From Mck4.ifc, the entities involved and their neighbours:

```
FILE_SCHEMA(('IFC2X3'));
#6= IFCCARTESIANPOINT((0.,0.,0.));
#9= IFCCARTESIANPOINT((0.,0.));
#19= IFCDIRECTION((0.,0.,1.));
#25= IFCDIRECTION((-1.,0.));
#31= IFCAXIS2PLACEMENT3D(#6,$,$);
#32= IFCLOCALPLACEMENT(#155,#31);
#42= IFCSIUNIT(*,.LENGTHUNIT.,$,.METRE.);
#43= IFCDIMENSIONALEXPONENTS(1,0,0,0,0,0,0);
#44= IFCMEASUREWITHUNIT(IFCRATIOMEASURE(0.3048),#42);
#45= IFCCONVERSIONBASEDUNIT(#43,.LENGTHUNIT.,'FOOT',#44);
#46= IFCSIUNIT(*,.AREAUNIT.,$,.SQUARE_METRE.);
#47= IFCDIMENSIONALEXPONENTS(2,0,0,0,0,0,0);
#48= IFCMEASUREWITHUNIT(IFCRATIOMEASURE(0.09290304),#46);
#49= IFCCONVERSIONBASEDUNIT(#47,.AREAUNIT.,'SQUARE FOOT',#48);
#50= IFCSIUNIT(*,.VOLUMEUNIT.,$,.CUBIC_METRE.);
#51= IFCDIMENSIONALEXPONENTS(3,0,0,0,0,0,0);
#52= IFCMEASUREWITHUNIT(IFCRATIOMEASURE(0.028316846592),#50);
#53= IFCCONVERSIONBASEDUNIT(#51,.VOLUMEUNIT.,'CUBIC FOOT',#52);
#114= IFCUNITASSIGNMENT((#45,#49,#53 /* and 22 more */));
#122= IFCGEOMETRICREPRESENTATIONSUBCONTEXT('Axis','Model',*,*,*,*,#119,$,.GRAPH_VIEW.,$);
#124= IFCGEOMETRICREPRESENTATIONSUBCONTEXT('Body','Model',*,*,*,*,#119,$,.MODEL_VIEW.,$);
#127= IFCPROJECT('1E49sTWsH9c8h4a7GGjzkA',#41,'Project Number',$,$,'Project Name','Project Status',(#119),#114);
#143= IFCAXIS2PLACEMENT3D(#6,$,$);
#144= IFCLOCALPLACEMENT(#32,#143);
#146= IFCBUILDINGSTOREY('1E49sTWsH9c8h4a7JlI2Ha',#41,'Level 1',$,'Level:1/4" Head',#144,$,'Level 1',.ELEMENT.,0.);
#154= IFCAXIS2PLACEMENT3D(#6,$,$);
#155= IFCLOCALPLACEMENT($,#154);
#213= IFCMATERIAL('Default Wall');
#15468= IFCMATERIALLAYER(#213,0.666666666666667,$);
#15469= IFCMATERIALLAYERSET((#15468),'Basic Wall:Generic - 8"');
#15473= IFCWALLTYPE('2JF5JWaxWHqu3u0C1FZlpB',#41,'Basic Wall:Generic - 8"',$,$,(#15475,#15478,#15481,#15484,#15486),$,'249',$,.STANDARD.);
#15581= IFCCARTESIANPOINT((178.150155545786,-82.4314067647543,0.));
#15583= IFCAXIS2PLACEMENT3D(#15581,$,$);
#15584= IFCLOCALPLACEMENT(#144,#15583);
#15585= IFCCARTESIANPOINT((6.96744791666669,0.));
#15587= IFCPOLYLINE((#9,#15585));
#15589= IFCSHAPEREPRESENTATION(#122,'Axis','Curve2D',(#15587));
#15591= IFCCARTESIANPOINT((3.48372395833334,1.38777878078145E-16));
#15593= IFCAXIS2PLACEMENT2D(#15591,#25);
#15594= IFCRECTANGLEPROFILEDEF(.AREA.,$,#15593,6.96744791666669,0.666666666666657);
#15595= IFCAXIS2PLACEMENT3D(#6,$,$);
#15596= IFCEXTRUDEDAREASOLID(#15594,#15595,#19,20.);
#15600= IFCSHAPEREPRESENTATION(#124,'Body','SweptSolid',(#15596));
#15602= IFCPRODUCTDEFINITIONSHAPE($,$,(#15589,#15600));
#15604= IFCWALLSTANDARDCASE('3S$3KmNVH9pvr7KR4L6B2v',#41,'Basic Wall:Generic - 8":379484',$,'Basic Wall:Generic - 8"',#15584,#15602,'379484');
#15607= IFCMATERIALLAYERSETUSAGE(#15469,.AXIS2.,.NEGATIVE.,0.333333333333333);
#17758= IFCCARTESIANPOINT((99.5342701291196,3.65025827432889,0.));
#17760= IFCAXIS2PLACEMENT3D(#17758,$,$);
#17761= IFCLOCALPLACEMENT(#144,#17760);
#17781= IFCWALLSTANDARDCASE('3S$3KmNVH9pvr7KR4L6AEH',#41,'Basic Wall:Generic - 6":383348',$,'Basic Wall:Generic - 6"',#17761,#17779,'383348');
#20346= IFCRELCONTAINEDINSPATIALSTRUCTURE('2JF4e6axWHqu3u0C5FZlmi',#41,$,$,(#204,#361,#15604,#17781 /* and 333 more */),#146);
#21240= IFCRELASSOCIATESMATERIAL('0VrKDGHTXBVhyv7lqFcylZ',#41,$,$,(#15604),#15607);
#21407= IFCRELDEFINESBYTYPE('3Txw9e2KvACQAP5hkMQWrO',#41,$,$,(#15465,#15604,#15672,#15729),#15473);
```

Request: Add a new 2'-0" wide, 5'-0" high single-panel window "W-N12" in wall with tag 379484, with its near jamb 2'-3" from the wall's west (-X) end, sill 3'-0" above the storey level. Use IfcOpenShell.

```python
import numpy as np
import ifcopenshell
import ifcopenshell.api.feature
import ifcopenshell.api.geometry
import ifcopenshell.api.root
import ifcopenshell.api.spatial
import ifcopenshell.api.type
import ifcopenshell.geom
import ifcopenshell.util.element
import ifcopenshell.util.placement
import ifcopenshell.util.representation
import ifcopenshell.util.shape
import ifcopenshell.util.unit

model = ifcopenshell.open("Mck4.ifc")
unit_scale = ifcopenshell.util.unit.calculate_unit_scale(model)
settings = ifcopenshell.geom.settings()


def volume(element):
    """Net volume in cubic metres, openings subtracted."""
    shape = ifcopenshell.geom.create_shape(settings, element)
    return ifcopenshell.util.shape.get_volume(shape.geometry)


wall = model.by_id(15604)
storey = ifcopenshell.util.element.get_container(wall, ifc_class="IfcBuildingStorey")
context = ifcopenshell.util.representation.get_context(model, "Model", "Body", "MODEL_VIEW")
before = volume(wall)

width, height, from_end, sill = 0.6096, 1.524, 0.6858, 0.9144  # metres

# The wall runs along its own X axis, and the end named is its -X end.
wall_shape = ifcopenshell.geom.create_shape(settings, wall)
x, y, z = ifcopenshell.util.shape.get_vertices(wall_shape.geometry).T
start = x.min() + from_end
face, thickness = float(y.min()), float(y.max() - y.min())
wall_matrix = ifcopenshell.util.placement.get_local_placement(wall.ObjectPlacement)
level = ifcopenshell.util.placement.get_local_placement(storey.ObjectPlacement)[2, 3]


def in_wall(x, y):
    """Placement at x, y metres in the wall's axes, at sill height."""
    matrix = wall_matrix.copy()
    matrix[:, 3] = wall_matrix @ np.array([x / unit_scale, y / unit_scale, 0.0, 1.0])
    matrix[2, 3] = level + sill / unit_scale
    return matrix


# Opening: a box that overshoots both wall faces by 50 mm.
opening = ifcopenshell.api.root.create_entity(model, ifc_class="IfcOpeningElement")
box = ifcopenshell.api.geometry.add_wall_representation(
    model, context=context, length=width, height=height, thickness=thickness + 0.1
)
ifcopenshell.api.geometry.assign_representation(model, product=opening, representation=box)
ifcopenshell.api.geometry.edit_object_placement(model, product=opening, matrix=in_wall(start, face - 0.05), is_si=False)
ifcopenshell.api.feature.add_feature(model, feature=opening, element=wall)

window = ifcopenshell.api.root.create_entity(model, ifc_class="IfcWindow", name="W-N12")
window.OverallWidth, window.OverallHeight = width / unit_scale, height / unit_scale
body = ifcopenshell.api.geometry.add_window_representation(
    model,
    context=context,
    overall_width=window.OverallWidth,
    overall_height=window.OverallHeight,
    partition_type="SINGLE_PANEL",
)
ifcopenshell.api.geometry.assign_representation(model, product=window, representation=body)
ifcopenshell.api.spatial.assign_container(model, products=[window], relating_structure=storey)
fills = ifcopenshell.api.feature.add_filling(model, opening=opening, element=window)
fills.OwnerHistory = window.OwnerHistory  # required in IFC2X3

# IFC2X3 keeps the operation on the window style.
style = ifcopenshell.api.root.create_entity(model, ifc_class="IfcWindowStyle", name="W-N12")
style.OperationType, style.ConstructionType = "SINGLE_PANEL", "NOTDEFINED"
style.ParameterTakesPrecedence = style.Sizeable = False
ifcopenshell.api.type.assign_type(model, related_objects=[window], relating_type=style)

# Centre the window in the wall's thickness.
ifcopenshell.api.geometry.edit_object_placement(model, product=window, matrix=in_wall(start, face), is_si=False)
window_shape = ifcopenshell.geom.create_shape(settings, window)
depth = ifcopenshell.util.shape.get_vertices(window_shape.geometry)[:, 1]
offset = face + thickness / 2 - (depth.min() + depth.max()) / 2
ifcopenshell.api.geometry.edit_object_placement(model, product=window, matrix=in_wall(start, offset), is_si=False)

after = volume(wall)

print(f"wall volume {before:.3f} -> {after:.3f} m3")

model.write("Mck4_updated.ifc")
```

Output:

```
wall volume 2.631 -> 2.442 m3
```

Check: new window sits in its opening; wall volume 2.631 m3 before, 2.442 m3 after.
